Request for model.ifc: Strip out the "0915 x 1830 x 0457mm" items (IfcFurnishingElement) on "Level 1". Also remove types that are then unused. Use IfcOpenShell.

First a look at what the model holds.

```python
import ifcopenshell
import ifcopenshell.util.element

model = ifcopenshell.open("model.ifc")
print(model.schema)
storey = next(s for s in model.by_type("IfcBuildingStorey") if s.Name == "Level 1")
furniture = [e for e in ifcopenshell.util.element.get_decomposition(storey) if e.is_a("IfcFurnishingElement")]
seen = {}
for e in furniture:
    element_type = ifcopenshell.util.element.get_type(e)
    name = element_type.Name if element_type not in (None, e) else None
    seen[name] = seen.get(name, 0) + 1
for name, count in sorted(seen.items(), key=str):
    print(count, "x", name)
```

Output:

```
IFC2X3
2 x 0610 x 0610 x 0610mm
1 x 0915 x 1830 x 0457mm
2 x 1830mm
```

```python
import ifcopenshell
import ifcopenshell.api.root
import ifcopenshell.util.element

model = ifcopenshell.open("model.ifc")

storey = next(s for s in model.by_type("IfcBuildingStorey") if s.Name == "Level 1")
furniture = [e for e in ifcopenshell.util.element.get_decomposition(storey) if e.is_a("IfcFurnishingElement")]
targets = [e for e in furniture if (t := ifcopenshell.util.element.get_type(e)) not in (None, e) and t.Name == "0915 x 1830 x 0457mm"]
types = {ifcopenshell.util.element.get_type(e) for e in targets} - {None, *targets}

for e in targets:
    ifcopenshell.api.root.remove_product(model, product=e)
print(len(targets), "removed")

unused = [t for t in types if not ifcopenshell.util.element.get_types(t)]
for t in unused:
    ifcopenshell.api.root.remove_product(model, product=t)
print(len(unused), "unused types removed")

model.write("model_v2.ifc")
```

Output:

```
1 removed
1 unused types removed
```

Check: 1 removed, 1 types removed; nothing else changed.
